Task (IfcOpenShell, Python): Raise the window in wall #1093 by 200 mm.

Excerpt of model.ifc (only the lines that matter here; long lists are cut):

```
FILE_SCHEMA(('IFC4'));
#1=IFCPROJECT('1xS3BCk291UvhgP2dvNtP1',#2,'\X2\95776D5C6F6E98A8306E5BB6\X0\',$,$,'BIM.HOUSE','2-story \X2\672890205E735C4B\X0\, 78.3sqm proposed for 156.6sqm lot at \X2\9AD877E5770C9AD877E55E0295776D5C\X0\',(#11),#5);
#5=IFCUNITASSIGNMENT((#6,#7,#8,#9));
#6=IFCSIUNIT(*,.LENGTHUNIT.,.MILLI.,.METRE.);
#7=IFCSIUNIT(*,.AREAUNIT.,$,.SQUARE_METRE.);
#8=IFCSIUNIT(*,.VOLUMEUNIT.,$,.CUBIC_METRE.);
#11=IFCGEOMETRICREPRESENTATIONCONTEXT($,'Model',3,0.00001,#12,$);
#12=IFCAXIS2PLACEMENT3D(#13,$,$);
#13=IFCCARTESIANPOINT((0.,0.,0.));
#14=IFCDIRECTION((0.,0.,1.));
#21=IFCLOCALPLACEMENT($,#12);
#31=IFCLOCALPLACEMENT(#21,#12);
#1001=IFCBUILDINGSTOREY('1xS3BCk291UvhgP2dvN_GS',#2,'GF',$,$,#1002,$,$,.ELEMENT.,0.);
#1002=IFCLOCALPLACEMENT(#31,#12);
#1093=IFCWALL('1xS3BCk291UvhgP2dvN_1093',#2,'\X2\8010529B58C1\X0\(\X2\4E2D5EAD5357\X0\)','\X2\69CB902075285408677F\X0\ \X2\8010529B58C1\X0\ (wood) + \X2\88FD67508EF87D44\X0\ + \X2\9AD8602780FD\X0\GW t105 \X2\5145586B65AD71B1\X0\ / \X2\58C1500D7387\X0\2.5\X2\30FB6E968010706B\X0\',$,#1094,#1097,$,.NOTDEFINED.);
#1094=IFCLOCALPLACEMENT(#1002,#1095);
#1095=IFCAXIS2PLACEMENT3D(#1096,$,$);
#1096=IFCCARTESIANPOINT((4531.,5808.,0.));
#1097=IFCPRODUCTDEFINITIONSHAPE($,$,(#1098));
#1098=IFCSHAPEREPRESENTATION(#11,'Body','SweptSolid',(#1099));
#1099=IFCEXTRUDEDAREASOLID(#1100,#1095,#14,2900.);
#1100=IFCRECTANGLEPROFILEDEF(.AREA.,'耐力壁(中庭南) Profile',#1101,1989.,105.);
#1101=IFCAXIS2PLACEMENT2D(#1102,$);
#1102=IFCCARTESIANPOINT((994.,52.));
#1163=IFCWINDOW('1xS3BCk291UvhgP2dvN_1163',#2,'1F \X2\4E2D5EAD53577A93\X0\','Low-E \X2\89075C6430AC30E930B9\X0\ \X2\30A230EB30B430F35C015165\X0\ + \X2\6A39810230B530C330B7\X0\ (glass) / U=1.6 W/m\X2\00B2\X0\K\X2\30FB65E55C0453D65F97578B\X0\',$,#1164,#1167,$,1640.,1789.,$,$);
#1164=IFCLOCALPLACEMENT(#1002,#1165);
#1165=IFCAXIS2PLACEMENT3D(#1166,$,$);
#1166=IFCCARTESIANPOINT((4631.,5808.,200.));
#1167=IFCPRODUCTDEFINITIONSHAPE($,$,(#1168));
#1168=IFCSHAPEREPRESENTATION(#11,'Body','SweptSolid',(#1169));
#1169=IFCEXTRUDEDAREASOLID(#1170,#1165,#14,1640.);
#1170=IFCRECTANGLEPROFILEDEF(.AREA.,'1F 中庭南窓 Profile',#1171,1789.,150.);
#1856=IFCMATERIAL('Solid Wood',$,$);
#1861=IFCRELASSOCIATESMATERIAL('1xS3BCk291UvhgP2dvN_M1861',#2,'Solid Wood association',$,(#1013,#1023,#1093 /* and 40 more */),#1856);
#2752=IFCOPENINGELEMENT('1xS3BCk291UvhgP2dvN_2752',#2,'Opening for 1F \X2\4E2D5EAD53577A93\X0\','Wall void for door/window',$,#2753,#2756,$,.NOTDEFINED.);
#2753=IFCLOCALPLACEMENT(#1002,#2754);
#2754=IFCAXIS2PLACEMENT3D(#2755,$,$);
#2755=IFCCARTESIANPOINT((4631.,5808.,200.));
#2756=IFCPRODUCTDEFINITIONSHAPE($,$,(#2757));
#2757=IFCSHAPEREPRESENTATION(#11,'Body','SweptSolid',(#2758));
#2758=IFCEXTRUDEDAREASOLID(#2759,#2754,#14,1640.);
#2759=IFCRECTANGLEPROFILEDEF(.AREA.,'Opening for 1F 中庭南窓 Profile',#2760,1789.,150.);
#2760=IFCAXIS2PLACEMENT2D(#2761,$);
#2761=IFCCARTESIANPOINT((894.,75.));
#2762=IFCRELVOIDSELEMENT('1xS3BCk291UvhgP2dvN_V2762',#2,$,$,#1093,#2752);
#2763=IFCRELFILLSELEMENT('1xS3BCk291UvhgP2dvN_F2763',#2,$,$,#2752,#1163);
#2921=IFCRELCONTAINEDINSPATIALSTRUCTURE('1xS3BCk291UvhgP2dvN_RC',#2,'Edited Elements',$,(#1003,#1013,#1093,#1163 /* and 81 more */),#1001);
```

```python
import numpy as np
import ifcopenshell
import ifcopenshell.api.geometry
import ifcopenshell.util.placement
import ifcopenshell.util.unit

model = ifcopenshell.open("model.ifc")
unit_scale = ifcopenshell.util.unit.calculate_unit_scale(model)

window = model.by_id(1163)
opening = window.FillsVoids[0].RelatingOpeningElement
dz = 0.2 / unit_scale

shift = np.array([0.0, 0.0, dz])
# The window is not placed relative to its opening, so move both.
for product in (opening, window):
    matrix = ifcopenshell.util.placement.get_local_placement(product.ObjectPlacement)
    matrix[:3, 3] += shift
    ifcopenshell.api.geometry.edit_object_placement(model, product=product, matrix=matrix, is_si=False)

print(f"moved by {dz * unit_scale:+.3f} m")

model.write("model_updated.ifc")
```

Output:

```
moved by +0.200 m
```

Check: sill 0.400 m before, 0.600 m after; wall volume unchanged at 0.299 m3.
